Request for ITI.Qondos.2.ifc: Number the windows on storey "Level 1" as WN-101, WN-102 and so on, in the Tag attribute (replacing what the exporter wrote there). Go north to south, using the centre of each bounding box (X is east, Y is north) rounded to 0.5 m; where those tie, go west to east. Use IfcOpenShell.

First a look at what the model holds.

```python
import ifcopenshell
import ifcopenshell.util.element
import ifcopenshell.util.placement

model = ifcopenshell.open("ITI.Qondos.2.ifc")
print(model.schema)
storey = next(s for s in model.by_type("IfcBuildingStorey") if s.Name == "Level 1")
windows = [e for e in ifcopenshell.util.element.get_decomposition(storey) if e.is_a("IfcWindow")]
for e in sorted(windows, key=lambda e: e.id()):
    origin = ifcopenshell.util.placement.get_local_placement(e.ObjectPlacement)[:3, 3]
    print(e.id(), e.Tag, e.Name, origin.round(2) + 0.0, sep=" | ")
```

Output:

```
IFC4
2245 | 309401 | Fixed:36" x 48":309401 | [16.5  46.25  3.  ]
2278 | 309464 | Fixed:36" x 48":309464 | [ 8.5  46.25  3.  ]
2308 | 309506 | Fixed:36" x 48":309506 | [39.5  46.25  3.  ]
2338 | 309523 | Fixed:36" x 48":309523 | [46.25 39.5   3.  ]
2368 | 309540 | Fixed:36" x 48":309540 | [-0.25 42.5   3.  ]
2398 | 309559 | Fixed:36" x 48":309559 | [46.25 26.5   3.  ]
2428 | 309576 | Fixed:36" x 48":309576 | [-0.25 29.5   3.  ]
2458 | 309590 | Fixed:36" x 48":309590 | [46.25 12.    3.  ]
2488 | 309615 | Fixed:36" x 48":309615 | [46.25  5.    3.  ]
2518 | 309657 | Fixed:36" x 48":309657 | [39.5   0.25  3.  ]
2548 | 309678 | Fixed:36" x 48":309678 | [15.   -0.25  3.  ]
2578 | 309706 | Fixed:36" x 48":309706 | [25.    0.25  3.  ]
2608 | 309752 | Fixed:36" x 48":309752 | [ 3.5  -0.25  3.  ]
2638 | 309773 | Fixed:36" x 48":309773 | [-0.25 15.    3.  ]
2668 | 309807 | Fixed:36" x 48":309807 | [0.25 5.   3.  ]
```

```python
import ifcopenshell
import ifcopenshell.geom
import ifcopenshell.util.element
import ifcopenshell.util.shape

model = ifcopenshell.open("ITI.Qondos.2.ifc")
settings = ifcopenshell.geom.settings()
settings.set("use-world-coords", True)


def centre(element):
    shape = ifcopenshell.geom.create_shape(settings, element)
    return ifcopenshell.util.shape.get_bbox_centroid(shape.geometry)


storey = next(s for s in model.by_type("IfcBuildingStorey") if s.Name == "Level 1")
windows = [e for e in ifcopenshell.util.element.get_decomposition(storey) if e.is_a("IfcWindow")]

# Insertion points can sit at a corner or the storey origin, so sort by the geometry (in metres).
centres = {e: centre(e) for e in windows}
windows.sort(key=lambda e: (-round(centres[e][1] / 0.5), centres[e][0]))

for i, e in enumerate(windows, start=1):
    number = f"WN-1{i:02d}"
    e.Tag = number
    print(e.id(), number)

model.write("ITI.Qondos.2_v2.ifc")
```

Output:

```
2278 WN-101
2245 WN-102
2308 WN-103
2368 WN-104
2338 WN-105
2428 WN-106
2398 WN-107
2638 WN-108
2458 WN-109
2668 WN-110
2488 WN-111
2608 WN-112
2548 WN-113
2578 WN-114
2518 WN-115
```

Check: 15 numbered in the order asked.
